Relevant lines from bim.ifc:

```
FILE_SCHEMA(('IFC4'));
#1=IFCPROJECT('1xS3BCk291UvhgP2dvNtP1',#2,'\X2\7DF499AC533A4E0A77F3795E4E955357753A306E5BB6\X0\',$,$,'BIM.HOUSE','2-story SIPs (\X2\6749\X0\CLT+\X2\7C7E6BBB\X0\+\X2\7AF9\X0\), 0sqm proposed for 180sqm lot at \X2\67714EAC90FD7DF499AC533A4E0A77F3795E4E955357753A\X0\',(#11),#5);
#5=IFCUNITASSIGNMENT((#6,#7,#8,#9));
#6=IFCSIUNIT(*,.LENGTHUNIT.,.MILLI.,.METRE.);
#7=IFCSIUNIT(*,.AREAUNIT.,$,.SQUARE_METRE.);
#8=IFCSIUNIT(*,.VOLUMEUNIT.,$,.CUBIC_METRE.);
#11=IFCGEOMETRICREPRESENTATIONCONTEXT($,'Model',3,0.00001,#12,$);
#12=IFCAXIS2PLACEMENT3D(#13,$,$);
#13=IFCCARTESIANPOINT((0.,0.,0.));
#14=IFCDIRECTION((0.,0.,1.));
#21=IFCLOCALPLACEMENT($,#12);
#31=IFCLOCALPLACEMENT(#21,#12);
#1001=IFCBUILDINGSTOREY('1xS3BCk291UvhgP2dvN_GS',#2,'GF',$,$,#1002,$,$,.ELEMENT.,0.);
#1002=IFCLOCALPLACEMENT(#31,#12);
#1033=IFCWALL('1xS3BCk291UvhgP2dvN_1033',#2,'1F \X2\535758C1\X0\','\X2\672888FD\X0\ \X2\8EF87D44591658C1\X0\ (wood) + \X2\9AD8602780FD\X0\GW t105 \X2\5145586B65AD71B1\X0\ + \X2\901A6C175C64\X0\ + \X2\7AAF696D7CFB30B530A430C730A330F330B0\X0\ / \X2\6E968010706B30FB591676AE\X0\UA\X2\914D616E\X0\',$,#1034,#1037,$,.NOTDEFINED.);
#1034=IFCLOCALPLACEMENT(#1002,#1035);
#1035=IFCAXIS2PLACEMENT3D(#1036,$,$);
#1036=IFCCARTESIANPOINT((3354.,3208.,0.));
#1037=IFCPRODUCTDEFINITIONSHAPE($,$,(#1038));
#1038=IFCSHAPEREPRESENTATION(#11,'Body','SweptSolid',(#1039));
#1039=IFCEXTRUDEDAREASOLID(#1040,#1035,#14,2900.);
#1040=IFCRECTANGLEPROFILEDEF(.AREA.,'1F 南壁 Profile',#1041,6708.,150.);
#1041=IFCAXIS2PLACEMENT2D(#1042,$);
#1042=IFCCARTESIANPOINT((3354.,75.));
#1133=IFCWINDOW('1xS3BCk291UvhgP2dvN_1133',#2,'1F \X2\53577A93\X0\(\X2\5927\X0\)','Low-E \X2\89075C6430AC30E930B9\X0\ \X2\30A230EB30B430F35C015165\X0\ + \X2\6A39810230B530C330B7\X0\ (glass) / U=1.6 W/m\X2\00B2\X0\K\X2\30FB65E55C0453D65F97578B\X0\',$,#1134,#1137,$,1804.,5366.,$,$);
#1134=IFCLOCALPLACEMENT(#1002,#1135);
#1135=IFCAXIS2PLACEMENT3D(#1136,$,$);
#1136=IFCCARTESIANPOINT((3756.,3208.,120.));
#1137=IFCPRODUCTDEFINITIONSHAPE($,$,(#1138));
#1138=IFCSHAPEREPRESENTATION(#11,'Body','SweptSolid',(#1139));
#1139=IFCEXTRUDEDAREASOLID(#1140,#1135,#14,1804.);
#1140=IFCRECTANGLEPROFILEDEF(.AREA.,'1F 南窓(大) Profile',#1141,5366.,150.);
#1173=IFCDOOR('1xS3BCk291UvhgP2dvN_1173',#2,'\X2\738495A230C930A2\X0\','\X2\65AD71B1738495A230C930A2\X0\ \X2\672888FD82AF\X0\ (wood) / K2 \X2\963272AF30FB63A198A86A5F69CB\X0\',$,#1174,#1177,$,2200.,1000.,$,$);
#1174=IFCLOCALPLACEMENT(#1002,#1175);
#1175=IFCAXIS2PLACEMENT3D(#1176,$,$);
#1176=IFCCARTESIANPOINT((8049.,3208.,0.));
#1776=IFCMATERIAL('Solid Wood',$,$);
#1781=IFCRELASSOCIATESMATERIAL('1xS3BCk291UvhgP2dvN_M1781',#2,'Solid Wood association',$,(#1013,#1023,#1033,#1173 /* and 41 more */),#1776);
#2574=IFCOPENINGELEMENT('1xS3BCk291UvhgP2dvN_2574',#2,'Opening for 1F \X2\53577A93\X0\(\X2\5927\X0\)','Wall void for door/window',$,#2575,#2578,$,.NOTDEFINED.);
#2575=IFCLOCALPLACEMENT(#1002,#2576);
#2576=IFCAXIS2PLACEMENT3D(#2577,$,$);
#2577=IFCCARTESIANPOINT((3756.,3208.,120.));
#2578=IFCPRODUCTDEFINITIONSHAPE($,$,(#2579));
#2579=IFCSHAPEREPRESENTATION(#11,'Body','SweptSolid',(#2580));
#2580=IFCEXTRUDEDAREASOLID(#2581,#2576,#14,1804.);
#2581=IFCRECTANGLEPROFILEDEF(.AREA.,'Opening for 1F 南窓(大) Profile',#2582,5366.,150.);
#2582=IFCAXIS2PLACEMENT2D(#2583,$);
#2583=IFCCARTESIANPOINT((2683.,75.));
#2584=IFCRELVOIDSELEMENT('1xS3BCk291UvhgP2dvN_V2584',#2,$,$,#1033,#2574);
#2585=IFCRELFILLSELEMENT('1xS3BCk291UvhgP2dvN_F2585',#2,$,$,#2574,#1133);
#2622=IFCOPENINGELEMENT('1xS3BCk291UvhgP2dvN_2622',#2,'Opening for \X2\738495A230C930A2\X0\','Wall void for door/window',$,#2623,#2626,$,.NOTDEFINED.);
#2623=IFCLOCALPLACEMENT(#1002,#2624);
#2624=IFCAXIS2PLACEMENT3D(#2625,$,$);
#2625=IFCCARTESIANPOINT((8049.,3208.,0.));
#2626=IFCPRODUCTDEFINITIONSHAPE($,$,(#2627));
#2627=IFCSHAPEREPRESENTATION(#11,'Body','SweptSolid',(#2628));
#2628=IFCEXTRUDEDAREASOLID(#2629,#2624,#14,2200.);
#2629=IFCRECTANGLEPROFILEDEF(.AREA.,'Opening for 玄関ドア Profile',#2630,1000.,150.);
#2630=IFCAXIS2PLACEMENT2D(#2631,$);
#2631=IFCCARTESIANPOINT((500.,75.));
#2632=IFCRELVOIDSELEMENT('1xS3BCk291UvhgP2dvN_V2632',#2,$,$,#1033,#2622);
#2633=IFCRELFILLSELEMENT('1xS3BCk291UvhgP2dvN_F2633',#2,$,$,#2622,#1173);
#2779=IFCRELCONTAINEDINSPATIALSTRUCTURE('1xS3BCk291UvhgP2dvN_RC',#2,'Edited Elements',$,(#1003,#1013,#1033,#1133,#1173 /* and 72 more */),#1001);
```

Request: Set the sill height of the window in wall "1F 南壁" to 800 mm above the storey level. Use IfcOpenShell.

```python
import numpy as np
import ifcopenshell
import ifcopenshell.api.geometry
import ifcopenshell.geom
import ifcopenshell.util.element
import ifcopenshell.util.placement
import ifcopenshell.util.shape
import ifcopenshell.util.unit

model = ifcopenshell.open("bim.ifc")
unit_scale = ifcopenshell.util.unit.calculate_unit_scale(model)

window = model.by_guid("1xS3BCk291UvhgP2dvN_1133")
opening = window.FillsVoids[0].RelatingOpeningElement
storey = ifcopenshell.util.element.get_container(window, ifc_class="IfcBuildingStorey")
level = ifcopenshell.util.placement.get_local_placement(storey.ObjectPlacement)[2, 3]

# The opening's origin need not be at the sill, so measure its lowest point.
shape = ifcopenshell.geom.create_shape(ifcopenshell.geom.settings(), opening)
bottom = ifcopenshell.util.shape.get_shape_bottom_elevation(shape, shape.geometry) / unit_scale
dz = level + 800.0 - bottom

shift = np.array([0.0, 0.0, dz])
# The window is not placed relative to its opening, so move both.
for product in (opening, window):
    matrix = ifcopenshell.util.placement.get_local_placement(product.ObjectPlacement)
    matrix[:3, 3] += shift
    ifcopenshell.api.geometry.edit_object_placement(model, product=product, matrix=matrix, is_si=False)

print(f"moved by {dz * unit_scale:+.3f} m")

model.write("bim_v2.ifc")
```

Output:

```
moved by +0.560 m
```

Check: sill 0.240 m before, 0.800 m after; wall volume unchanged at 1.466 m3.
